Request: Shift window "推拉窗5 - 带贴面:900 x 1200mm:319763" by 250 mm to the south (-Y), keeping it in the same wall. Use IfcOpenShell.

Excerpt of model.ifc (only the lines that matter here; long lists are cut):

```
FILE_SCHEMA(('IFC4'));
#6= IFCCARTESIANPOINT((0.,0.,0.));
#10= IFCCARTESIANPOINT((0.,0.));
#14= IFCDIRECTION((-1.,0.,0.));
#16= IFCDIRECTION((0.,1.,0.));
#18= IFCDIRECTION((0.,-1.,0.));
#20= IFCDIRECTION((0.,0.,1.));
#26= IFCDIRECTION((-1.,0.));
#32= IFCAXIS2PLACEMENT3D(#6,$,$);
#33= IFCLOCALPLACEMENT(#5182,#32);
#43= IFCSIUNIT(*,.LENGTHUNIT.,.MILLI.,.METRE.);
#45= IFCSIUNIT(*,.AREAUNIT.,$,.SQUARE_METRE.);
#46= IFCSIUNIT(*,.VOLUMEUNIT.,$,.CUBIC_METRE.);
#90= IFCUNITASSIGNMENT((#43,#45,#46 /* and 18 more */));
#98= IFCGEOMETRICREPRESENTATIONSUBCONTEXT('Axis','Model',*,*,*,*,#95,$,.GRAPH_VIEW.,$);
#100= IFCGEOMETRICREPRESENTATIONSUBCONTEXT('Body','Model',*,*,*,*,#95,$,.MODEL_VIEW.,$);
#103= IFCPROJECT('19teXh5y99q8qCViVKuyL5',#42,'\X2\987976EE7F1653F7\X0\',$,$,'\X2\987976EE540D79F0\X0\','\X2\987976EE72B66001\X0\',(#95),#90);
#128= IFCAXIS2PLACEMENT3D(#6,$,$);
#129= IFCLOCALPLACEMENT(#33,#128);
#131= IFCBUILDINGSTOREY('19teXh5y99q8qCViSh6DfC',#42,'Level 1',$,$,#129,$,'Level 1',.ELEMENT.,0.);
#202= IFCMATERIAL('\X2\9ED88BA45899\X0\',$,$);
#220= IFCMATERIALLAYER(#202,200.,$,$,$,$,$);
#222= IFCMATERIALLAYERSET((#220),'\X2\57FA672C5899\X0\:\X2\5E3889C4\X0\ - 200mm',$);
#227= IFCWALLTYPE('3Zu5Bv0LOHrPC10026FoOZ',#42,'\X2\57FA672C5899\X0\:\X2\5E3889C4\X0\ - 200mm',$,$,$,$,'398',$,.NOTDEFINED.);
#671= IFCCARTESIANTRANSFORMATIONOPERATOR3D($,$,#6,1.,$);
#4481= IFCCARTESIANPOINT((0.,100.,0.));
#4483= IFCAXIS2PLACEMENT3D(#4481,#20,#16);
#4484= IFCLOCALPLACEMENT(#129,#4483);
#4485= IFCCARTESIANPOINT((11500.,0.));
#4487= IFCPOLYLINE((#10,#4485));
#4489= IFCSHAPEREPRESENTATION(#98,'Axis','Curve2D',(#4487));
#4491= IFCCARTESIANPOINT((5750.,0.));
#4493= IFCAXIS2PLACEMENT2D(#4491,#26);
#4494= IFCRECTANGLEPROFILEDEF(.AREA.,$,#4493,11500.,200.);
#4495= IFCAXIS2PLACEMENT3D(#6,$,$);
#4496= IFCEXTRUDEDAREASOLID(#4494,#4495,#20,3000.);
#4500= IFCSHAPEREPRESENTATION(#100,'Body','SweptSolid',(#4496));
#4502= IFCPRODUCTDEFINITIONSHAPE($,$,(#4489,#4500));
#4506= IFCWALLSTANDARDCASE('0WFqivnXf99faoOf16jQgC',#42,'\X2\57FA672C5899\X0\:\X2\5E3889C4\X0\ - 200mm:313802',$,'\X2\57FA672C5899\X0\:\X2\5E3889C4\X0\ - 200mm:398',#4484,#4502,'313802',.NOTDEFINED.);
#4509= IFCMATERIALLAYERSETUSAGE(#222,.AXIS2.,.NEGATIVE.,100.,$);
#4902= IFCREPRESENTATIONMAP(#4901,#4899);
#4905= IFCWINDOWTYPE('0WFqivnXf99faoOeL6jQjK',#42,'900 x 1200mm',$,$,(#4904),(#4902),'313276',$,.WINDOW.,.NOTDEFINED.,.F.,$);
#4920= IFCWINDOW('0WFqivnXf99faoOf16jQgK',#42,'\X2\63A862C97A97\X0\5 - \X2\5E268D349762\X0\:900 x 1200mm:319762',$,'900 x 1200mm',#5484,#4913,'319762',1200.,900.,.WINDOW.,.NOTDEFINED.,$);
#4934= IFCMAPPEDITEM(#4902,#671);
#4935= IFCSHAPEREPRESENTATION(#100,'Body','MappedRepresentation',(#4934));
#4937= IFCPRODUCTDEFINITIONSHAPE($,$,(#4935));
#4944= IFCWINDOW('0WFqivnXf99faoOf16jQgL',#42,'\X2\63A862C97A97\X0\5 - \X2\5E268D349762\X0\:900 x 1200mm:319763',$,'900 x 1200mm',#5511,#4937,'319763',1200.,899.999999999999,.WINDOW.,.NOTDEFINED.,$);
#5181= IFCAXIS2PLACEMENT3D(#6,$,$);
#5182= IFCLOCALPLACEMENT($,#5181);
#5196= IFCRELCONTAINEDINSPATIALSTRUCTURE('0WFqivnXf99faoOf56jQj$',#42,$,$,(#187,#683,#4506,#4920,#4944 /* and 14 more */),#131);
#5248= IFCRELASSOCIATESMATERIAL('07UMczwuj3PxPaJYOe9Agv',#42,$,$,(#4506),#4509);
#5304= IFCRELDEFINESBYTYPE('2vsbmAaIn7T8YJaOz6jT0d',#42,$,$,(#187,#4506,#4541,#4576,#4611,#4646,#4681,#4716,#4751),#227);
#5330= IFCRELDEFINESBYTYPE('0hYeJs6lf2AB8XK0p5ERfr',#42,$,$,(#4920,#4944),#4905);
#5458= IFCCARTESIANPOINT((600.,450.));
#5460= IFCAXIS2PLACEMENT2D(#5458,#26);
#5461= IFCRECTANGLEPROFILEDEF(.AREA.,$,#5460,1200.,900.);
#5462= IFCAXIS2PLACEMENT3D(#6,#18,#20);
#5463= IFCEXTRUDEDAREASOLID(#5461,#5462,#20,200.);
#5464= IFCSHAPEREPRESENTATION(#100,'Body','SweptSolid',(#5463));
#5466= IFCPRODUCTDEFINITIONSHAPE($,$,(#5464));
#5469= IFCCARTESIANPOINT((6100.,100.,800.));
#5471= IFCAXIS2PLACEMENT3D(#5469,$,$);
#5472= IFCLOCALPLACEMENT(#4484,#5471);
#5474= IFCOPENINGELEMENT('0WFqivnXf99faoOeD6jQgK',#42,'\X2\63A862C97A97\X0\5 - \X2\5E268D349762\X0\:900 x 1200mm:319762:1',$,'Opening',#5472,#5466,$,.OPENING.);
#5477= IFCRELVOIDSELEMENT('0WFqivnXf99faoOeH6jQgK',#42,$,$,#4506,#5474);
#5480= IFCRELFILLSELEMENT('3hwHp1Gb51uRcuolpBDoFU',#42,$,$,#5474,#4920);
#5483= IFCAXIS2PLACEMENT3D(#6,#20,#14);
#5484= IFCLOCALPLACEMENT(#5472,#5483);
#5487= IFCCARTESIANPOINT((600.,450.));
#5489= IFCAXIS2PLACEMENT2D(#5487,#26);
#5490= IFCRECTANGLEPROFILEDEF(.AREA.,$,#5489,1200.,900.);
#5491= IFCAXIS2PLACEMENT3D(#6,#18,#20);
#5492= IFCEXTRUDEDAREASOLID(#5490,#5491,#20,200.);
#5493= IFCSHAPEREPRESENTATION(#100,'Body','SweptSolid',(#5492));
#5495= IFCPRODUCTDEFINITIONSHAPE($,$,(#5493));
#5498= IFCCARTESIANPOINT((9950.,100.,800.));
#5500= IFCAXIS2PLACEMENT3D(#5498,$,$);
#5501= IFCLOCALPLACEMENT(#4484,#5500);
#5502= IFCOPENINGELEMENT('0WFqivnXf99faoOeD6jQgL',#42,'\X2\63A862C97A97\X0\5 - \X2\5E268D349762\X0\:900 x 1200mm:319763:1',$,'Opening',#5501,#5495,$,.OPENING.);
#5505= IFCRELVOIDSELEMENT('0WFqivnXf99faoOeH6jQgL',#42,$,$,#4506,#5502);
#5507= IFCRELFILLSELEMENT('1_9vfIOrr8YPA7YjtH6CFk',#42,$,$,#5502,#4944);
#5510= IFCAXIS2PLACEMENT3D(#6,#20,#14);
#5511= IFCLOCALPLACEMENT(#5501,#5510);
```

```python
import ifcopenshell
import ifcopenshell.api.geometry
import ifcopenshell.util.placement
import ifcopenshell.util.unit

model = ifcopenshell.open("model.ifc")
unit_scale = ifcopenshell.util.unit.calculate_unit_scale(model)

window = model.by_guid("0WFqivnXf99faoOf16jQgL")
opening = window.FillsVoids[0].RelatingOpeningElement
wall = opening.VoidsElements[0].RelatingBuildingElement

wall_matrix = ifcopenshell.util.placement.get_local_placement(wall.ObjectPlacement)
shift = wall_matrix[:3, 0] * -0.25 / unit_scale
before = ifcopenshell.util.placement.get_local_placement(window.ObjectPlacement)[:3, 3].copy()

# The window is placed relative to its opening, so it follows when the opening moves.
matrix = ifcopenshell.util.placement.get_local_placement(opening.ObjectPlacement)
matrix[:3, 3] += shift
ifcopenshell.api.geometry.edit_object_placement(
    model, product=opening, matrix=matrix, is_si=False, should_transform_children=True
)

after = ifcopenshell.util.placement.get_local_placement(window.ObjectPlacement)[:3, 3]
print("window moved by", (after - before).round(3) + 0.0)

model.write("model_updated.ifc")
```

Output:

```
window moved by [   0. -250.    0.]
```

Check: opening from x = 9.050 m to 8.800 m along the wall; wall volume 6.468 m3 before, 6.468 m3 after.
